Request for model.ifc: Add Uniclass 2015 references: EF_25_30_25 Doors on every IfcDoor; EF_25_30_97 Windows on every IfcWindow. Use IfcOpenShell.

First a look at what the model holds.

```python
import ifcopenshell

model = ifcopenshell.open("model.ifc")
print(model.schema)
print("classifications:", [c.Name for c in model.by_type("IfcClassification")])
for ifc_class in ("IfcDoor", "IfcRoof", "IfcStair", "IfcWall", "IfcWindow"):
    print(ifc_class, len(model.by_type(ifc_class)))
```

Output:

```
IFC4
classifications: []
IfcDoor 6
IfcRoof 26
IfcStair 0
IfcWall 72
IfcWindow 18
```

```python
import ifcopenshell
import ifcopenshell.api.classification

model = ifcopenshell.open("model.ifc")

system = ifcopenshell.api.classification.add_classification(model, classification="Uniclass 2015")

codes = {
    "IfcDoor": ("EF_25_30_25", "Doors"),
    "IfcWindow": ("EF_25_30_97", "Windows"),
}
for ifc_class, (code, name) in codes.items():
    products = model.by_type(ifc_class)
    ifcopenshell.api.classification.add_reference(
        model, products=products, classification=system, identification=code, name=name
    )
    print(code, len(products))

model.write("model_v2.ifc")
```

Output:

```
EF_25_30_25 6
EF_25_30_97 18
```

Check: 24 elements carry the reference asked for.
